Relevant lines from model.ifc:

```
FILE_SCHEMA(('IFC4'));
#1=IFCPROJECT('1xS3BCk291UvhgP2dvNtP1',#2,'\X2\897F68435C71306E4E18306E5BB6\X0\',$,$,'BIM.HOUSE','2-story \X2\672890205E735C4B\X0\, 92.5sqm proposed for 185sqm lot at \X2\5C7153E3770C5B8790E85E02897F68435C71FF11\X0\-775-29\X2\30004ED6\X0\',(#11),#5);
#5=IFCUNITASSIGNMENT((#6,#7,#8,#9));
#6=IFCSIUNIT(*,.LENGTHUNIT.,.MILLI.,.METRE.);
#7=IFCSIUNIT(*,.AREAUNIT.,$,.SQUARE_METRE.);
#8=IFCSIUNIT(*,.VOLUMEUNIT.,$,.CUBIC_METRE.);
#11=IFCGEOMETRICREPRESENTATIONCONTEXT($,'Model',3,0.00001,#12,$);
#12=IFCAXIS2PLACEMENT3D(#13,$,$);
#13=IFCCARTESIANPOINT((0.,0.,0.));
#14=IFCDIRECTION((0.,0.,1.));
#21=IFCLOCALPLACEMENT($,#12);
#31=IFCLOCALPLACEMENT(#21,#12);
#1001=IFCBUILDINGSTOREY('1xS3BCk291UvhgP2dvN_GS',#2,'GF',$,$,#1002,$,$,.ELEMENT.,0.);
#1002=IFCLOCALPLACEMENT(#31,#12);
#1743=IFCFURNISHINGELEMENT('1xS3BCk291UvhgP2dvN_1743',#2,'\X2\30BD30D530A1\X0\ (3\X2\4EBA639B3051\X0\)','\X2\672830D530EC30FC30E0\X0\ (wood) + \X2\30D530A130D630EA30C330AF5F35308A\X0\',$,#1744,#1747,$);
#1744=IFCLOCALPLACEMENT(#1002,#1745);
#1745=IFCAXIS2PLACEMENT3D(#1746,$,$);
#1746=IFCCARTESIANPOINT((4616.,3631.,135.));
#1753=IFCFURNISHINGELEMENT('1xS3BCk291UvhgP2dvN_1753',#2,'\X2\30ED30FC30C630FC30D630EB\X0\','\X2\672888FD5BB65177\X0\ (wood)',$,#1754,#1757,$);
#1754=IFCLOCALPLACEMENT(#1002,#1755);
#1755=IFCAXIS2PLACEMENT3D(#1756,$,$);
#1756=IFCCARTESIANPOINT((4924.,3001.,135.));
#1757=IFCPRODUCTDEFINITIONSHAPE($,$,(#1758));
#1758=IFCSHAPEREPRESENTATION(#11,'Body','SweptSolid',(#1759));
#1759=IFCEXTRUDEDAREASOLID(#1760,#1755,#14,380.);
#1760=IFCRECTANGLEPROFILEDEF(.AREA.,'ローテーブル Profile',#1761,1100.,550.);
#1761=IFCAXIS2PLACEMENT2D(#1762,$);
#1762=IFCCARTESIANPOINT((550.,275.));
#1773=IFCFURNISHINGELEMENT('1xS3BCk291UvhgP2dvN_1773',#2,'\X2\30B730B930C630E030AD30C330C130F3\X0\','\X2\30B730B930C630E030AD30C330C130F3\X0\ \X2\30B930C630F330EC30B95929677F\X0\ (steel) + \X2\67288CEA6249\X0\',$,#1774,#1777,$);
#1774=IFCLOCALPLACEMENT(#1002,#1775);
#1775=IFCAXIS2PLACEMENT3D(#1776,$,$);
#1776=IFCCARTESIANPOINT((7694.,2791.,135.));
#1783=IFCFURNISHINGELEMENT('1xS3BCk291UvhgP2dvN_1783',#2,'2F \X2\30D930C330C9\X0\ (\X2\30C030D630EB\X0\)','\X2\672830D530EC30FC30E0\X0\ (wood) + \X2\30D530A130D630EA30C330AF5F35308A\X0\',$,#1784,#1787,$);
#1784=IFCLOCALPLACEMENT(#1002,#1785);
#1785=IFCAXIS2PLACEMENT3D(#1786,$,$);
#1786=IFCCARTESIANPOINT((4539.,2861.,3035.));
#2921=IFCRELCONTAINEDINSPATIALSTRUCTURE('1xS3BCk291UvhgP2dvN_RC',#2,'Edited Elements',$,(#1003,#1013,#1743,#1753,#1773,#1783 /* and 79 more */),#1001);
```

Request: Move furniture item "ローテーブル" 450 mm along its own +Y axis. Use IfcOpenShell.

```python
import ifcopenshell
import ifcopenshell.api.geometry
import ifcopenshell.util.placement
import ifcopenshell.util.unit

model = ifcopenshell.open("model.ifc")
unit_scale = ifcopenshell.util.unit.calculate_unit_scale(model)

item = model.by_guid("1xS3BCk291UvhgP2dvN_1753")
matrix = ifcopenshell.util.placement.get_local_placement(item.ObjectPlacement)
matrix[:3, 3] += matrix[:3, 1] * 0.45 / unit_scale
ifcopenshell.api.geometry.edit_object_placement(model, product=item, matrix=matrix, is_si=False)

print(ifcopenshell.util.placement.get_local_placement(item.ObjectPlacement).round(3) + 0.0)

model.write("model-out.ifc")
```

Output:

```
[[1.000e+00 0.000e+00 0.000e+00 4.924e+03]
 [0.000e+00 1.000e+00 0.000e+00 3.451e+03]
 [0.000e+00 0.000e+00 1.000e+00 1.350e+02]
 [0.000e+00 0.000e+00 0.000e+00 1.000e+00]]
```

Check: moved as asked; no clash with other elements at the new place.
